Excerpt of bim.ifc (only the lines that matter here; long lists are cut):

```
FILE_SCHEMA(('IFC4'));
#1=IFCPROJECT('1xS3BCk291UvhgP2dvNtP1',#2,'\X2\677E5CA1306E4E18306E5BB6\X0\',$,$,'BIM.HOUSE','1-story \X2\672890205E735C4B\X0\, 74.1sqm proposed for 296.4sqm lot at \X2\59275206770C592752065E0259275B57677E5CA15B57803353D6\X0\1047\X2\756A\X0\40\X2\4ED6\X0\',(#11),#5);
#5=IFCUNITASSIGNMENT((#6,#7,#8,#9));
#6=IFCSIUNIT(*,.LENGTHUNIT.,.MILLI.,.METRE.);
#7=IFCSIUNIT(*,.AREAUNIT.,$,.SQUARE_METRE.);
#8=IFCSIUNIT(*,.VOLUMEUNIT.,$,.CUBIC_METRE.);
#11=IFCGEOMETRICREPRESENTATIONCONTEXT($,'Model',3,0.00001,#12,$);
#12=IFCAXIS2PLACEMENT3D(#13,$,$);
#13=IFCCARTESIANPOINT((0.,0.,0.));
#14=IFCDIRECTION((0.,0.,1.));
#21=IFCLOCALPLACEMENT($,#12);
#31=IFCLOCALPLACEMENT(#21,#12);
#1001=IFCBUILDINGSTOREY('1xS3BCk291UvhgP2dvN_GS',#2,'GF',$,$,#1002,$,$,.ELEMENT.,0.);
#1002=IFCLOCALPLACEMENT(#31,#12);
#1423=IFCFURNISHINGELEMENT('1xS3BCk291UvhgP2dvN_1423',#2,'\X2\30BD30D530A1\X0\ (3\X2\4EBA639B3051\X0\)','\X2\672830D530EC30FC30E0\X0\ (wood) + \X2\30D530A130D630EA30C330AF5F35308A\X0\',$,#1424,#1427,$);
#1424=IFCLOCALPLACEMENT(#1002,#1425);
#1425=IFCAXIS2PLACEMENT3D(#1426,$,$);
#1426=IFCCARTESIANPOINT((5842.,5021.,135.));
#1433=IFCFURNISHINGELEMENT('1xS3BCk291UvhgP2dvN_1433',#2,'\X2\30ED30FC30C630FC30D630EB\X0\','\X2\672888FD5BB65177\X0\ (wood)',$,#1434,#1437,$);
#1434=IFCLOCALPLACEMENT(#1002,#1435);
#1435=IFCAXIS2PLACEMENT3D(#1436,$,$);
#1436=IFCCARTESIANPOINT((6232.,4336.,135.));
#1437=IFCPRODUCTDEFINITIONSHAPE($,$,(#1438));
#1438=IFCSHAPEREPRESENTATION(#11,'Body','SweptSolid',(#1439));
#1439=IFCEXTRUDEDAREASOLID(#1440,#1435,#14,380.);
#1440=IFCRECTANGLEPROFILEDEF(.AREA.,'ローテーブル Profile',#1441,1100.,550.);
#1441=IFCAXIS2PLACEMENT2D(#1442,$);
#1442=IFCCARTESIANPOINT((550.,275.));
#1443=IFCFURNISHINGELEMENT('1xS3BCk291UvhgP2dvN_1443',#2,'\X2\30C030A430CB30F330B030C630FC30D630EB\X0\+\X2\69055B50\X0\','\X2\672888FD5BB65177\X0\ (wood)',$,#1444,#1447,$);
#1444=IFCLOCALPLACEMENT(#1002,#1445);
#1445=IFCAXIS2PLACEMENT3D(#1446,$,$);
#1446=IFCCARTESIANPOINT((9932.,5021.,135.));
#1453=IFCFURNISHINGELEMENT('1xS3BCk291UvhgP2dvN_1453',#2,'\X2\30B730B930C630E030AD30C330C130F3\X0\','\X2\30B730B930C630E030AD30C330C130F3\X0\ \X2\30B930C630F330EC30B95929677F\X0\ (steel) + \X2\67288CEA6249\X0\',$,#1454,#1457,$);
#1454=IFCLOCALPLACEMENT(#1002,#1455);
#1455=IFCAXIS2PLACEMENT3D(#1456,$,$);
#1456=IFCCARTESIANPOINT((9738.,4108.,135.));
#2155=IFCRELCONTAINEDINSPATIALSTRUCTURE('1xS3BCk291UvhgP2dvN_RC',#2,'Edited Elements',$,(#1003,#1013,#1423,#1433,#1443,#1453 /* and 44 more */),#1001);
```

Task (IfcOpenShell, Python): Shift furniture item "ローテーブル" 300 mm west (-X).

```python
import ifcopenshell
import ifcopenshell.api.geometry
import ifcopenshell.util.placement
import ifcopenshell.util.unit

model = ifcopenshell.open("bim.ifc")
unit_scale = ifcopenshell.util.unit.calculate_unit_scale(model)

item = model.by_guid("1xS3BCk291UvhgP2dvN_1433")
matrix = ifcopenshell.util.placement.get_local_placement(item.ObjectPlacement)
matrix[0, 3] -= 0.3 / unit_scale
ifcopenshell.api.geometry.edit_object_placement(model, product=item, matrix=matrix, is_si=False)

print(ifcopenshell.util.placement.get_local_placement(item.ObjectPlacement).round(3) + 0.0)

model.write("bim-out.ifc")
```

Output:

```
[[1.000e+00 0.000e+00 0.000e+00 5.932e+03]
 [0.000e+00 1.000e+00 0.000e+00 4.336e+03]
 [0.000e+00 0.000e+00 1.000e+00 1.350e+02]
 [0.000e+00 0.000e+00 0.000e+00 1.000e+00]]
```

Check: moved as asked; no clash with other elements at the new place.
